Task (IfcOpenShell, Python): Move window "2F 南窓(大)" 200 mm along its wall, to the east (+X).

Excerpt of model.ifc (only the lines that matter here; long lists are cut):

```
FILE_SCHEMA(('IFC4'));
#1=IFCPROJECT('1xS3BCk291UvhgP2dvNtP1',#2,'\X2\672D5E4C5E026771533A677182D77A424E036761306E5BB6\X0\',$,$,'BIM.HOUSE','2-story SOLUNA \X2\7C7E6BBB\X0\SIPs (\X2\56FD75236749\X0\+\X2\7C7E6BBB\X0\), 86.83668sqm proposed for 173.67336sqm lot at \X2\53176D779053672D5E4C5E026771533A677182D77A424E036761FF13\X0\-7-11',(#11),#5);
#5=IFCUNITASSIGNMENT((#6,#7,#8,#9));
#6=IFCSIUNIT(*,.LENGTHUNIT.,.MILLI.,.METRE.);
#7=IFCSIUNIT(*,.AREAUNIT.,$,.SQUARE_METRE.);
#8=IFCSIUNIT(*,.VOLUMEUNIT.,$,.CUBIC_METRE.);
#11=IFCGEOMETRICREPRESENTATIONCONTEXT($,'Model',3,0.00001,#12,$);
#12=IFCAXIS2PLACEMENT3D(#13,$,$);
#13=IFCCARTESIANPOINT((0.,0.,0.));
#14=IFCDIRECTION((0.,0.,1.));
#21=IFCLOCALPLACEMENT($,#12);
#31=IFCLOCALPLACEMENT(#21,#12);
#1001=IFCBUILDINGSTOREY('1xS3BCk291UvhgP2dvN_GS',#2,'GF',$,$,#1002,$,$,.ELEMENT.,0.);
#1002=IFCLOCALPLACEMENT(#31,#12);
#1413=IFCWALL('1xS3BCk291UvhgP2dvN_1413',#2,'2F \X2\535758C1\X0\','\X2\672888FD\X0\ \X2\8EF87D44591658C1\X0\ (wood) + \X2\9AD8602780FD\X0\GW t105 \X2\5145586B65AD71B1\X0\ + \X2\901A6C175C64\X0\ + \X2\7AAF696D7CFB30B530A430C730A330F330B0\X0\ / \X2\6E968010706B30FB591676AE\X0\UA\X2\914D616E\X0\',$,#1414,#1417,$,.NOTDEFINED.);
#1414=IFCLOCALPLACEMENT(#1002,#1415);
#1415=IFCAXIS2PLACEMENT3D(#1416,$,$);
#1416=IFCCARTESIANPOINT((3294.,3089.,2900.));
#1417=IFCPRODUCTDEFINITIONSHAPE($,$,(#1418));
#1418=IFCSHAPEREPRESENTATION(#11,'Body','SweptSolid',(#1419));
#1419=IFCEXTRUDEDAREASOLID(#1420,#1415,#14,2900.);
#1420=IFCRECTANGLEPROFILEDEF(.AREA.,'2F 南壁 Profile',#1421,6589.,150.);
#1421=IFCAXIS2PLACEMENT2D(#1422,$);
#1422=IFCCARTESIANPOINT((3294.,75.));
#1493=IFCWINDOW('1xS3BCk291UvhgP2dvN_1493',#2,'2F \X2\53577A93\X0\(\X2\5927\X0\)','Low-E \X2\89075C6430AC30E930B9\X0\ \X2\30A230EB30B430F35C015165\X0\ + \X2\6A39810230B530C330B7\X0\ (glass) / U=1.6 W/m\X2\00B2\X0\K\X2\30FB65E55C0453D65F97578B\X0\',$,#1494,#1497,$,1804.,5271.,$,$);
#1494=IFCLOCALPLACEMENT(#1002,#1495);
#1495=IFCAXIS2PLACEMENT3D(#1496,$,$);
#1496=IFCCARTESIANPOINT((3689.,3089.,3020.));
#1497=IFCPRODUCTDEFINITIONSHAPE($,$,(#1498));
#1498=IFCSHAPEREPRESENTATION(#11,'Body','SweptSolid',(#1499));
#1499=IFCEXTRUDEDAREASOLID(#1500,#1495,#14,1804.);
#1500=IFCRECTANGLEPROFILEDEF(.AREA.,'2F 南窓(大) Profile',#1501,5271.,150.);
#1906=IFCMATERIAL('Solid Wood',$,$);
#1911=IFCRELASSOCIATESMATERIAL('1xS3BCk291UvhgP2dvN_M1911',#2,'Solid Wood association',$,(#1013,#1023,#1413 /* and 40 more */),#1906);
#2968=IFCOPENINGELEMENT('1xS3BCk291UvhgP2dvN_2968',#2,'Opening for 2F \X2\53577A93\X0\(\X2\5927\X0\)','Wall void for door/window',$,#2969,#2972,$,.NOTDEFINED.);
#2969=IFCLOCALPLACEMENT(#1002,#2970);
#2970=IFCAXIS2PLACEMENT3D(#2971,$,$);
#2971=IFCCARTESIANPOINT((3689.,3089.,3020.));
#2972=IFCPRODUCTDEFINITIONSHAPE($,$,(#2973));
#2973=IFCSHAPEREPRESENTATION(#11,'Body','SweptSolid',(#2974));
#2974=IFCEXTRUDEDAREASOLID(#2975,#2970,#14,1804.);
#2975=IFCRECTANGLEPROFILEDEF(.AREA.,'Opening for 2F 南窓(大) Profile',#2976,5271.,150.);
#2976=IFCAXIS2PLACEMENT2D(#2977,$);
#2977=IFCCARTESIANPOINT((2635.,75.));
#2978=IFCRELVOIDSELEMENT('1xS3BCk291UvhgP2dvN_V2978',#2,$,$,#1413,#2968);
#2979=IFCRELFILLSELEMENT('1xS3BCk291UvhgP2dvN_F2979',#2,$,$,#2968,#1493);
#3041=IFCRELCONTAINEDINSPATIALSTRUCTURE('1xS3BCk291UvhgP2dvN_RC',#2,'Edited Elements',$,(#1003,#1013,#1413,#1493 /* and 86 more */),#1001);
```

```python
import ifcopenshell
import ifcopenshell.api.geometry
import ifcopenshell.util.placement
import ifcopenshell.util.unit

model = ifcopenshell.open("model.ifc")
unit_scale = ifcopenshell.util.unit.calculate_unit_scale(model)

window = model.by_guid("1xS3BCk291UvhgP2dvN_1493")
opening = window.FillsVoids[0].RelatingOpeningElement
wall = opening.VoidsElements[0].RelatingBuildingElement

wall_matrix = ifcopenshell.util.placement.get_local_placement(wall.ObjectPlacement)
shift = wall_matrix[:3, 0] * 0.2 / unit_scale
before = ifcopenshell.util.placement.get_local_placement(window.ObjectPlacement)[:3, 3].copy()

# The window is not placed relative to its opening, so move both.
for product in (opening, window):
    matrix = ifcopenshell.util.placement.get_local_placement(product.ObjectPlacement)
    matrix[:3, 3] += shift
    ifcopenshell.api.geometry.edit_object_placement(model, product=product, matrix=matrix, is_si=False)

after = ifcopenshell.util.placement.get_local_placement(window.ObjectPlacement)[:3, 3]
print("window moved by", (after - before).round(3) + 0.0)

model.write("model_edited.ifc")
```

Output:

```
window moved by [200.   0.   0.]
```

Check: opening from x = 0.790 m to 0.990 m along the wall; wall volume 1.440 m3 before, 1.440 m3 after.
